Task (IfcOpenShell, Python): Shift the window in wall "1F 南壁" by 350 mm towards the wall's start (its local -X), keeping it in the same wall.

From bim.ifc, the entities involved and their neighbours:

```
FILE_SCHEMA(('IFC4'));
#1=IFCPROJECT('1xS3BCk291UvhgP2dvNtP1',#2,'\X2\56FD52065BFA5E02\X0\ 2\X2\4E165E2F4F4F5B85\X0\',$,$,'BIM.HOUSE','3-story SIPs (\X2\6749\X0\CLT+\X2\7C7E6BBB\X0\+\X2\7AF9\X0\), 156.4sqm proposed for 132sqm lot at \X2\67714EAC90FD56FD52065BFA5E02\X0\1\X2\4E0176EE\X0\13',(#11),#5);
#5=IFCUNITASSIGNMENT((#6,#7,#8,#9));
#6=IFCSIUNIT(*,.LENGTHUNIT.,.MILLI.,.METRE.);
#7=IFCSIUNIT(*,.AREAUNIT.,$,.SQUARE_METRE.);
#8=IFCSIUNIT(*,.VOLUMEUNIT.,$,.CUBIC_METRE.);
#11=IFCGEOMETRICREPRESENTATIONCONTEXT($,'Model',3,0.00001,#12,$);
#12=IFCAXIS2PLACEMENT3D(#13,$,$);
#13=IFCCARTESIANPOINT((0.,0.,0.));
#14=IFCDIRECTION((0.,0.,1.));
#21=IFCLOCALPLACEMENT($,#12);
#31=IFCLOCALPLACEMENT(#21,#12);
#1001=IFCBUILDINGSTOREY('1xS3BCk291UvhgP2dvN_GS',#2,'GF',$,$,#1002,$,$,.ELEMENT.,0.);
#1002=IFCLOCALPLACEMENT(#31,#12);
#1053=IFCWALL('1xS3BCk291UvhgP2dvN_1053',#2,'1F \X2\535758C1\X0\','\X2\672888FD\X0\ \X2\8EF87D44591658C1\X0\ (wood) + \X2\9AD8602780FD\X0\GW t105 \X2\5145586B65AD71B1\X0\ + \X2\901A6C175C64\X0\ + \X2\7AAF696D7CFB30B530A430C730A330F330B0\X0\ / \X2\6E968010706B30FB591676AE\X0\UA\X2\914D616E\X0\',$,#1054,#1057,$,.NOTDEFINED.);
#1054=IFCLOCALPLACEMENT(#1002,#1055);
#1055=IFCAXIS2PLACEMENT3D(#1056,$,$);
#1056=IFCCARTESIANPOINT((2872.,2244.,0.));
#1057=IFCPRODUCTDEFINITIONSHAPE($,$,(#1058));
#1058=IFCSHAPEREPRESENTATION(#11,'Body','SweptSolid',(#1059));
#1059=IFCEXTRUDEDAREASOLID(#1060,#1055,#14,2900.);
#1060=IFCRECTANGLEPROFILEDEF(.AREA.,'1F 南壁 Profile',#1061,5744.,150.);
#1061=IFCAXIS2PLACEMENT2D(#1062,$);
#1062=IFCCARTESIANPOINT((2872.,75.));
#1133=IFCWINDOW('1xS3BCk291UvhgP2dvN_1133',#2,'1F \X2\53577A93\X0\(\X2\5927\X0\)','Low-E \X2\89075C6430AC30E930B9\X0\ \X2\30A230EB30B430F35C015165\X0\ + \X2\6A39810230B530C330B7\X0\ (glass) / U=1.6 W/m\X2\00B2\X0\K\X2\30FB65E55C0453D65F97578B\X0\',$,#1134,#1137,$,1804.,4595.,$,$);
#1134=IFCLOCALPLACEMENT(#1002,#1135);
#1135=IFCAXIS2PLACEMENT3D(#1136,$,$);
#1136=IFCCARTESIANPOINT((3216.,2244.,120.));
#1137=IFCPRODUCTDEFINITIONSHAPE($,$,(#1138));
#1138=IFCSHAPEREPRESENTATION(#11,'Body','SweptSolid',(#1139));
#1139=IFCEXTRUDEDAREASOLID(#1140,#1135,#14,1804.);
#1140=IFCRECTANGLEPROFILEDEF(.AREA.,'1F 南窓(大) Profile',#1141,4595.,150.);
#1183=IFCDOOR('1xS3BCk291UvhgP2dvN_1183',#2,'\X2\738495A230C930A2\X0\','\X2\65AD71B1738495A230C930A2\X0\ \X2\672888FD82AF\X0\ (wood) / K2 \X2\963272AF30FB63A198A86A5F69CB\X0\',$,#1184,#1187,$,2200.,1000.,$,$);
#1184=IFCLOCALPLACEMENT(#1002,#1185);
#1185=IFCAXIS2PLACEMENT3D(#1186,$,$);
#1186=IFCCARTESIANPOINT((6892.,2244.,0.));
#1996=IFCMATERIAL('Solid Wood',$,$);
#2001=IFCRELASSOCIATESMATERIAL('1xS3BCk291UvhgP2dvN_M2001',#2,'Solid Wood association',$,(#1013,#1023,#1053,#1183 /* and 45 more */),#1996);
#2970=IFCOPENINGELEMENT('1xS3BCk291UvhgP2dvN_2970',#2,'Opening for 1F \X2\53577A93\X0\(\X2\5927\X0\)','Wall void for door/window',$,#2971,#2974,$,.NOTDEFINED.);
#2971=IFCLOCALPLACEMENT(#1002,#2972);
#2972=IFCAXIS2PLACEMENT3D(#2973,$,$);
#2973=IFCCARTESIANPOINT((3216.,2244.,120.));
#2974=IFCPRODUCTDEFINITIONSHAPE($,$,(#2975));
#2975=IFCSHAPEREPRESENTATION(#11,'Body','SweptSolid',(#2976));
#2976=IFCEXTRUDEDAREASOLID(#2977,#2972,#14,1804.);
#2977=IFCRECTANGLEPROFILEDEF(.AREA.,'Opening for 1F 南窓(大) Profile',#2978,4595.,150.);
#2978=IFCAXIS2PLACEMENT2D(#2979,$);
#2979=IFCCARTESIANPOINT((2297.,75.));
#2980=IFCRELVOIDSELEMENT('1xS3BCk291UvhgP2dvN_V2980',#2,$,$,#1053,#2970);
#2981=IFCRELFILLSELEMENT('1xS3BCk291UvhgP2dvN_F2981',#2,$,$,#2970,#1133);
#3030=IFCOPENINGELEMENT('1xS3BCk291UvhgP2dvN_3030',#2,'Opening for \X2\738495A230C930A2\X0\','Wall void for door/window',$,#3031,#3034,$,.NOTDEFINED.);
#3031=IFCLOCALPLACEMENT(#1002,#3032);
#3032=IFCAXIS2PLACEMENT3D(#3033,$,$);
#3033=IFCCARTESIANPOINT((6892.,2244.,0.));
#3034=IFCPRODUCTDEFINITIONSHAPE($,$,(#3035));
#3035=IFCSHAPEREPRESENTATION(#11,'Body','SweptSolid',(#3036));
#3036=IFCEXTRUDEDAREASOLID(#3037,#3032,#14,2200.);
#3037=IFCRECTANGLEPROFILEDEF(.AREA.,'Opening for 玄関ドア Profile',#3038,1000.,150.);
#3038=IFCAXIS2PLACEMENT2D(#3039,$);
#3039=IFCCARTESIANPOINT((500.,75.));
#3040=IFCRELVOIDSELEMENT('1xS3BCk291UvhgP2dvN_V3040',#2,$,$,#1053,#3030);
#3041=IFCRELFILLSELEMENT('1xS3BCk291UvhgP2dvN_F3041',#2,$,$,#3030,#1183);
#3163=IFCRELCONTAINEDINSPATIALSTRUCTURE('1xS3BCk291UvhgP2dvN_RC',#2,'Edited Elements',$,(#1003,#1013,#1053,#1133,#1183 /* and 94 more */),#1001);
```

```python
import ifcopenshell
import ifcopenshell.api.geometry
import ifcopenshell.util.placement
import ifcopenshell.util.unit

model = ifcopenshell.open("bim.ifc")
unit_scale = ifcopenshell.util.unit.calculate_unit_scale(model)

window = model.by_id(1133)
opening = window.FillsVoids[0].RelatingOpeningElement
wall = opening.VoidsElements[0].RelatingBuildingElement

wall_matrix = ifcopenshell.util.placement.get_local_placement(wall.ObjectPlacement)
shift = wall_matrix[:3, 0] * -0.35 / unit_scale
before = ifcopenshell.util.placement.get_local_placement(window.ObjectPlacement)[:3, 3].copy()

# The window is not placed relative to its opening, so move both.
for product in (opening, window):
    matrix = ifcopenshell.util.placement.get_local_placement(product.ObjectPlacement)
    matrix[:3, 3] += shift
    ifcopenshell.api.geometry.edit_object_placement(model, product=product, matrix=matrix, is_si=False)

after = ifcopenshell.util.placement.get_local_placement(window.ObjectPlacement)[:3, 3]
print("window moved by", (after - before).round(3) + 0.0)

model.write("bim-out.ifc")
```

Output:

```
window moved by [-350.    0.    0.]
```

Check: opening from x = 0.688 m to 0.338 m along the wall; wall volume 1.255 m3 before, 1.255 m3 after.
